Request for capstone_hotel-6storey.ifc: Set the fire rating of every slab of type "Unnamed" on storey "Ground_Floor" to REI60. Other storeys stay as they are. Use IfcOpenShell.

First a look at what the model holds.

```python
import ifcopenshell
import ifcopenshell.util.element

model = ifcopenshell.open("capstone_hotel-6storey.ifc")
print(model.schema)
storey = next(s for s in model.by_type("IfcBuildingStorey") if s.Name == "Ground_Floor")
slabs = [e for e in ifcopenshell.util.element.get_decomposition(storey) if e.is_a("IfcSlab")]
seen = {}
for e in slabs:
    element_type = ifcopenshell.util.element.get_type(e)
    key = (element_type.Name if element_type != e and element_type else None, ifcopenshell.util.element.get_pset(e, "Pset_SlabCommon", "FireRating"))
    seen[key] = seen.get(key, 0) + 1
for (name, value), count in sorted(seen.items(), key=str):
    print(count, "x", name, "|", value)
```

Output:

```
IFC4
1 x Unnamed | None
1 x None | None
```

```python
import ifcopenshell
import ifcopenshell.api.pset
import ifcopenshell.util.element

model = ifcopenshell.open("capstone_hotel-6storey.ifc")

storey = next(s for s in model.by_type("IfcBuildingStorey") if s.Name == "Ground_Floor")
slabs = [e for e in ifcopenshell.util.element.get_decomposition(storey) if e.is_a("IfcSlab")]

count = 0
for e in slabs:
    element_type = ifcopenshell.util.element.get_type(e)
    if element_type in (None, e) or element_type.Name != "Unnamed":
        continue
    # add_pset returns the element's existing set when there is one.
    pset = ifcopenshell.api.pset.add_pset(model, product=e, name="Pset_SlabCommon")
    ifcopenshell.api.pset.edit_pset(model, pset=pset, properties={"FireRating": "REI60"})
    count += 1

print(count, "slabs updated")

model.write("capstone_hotel-6storey-out.ifc")
```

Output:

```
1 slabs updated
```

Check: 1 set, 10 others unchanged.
